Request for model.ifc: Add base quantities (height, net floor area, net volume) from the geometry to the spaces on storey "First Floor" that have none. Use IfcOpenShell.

First a look at what the model holds.

```python
import ifcopenshell
import ifcopenshell.util.element
import ifcopenshell.util.unit

model = ifcopenshell.open("model.ifc")
print(model.schema)
for unit_type in ("LENGTHUNIT", "AREAUNIT", "VOLUMEUNIT"):
    print(unit_type, ifcopenshell.util.unit.calculate_unit_scale(model, unit_type))
storey = next(s for s in model.by_type("IfcBuildingStorey") if s.Name == "First Floor")
spaces = [e for e in ifcopenshell.util.element.get_decomposition(storey) if e.is_a("IfcSpace")]
for e in sorted(spaces, key=lambda e: e.id()):
    print(e.id(), e.is_a(), e.Name, list(ifcopenshell.util.element.get_psets(e, qtos_only=True)), sep=" | ")
```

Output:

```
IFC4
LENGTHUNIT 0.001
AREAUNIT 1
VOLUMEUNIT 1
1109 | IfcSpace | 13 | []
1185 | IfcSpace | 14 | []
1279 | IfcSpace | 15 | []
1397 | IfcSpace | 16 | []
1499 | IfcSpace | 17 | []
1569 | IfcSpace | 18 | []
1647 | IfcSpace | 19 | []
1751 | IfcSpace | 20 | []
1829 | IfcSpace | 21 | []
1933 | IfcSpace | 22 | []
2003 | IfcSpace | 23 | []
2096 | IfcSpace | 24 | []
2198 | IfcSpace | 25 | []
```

```python
import ifcopenshell
import ifcopenshell.api.pset
import ifcopenshell.geom
import ifcopenshell.util.element
import ifcopenshell.util.shape
import ifcopenshell.util.unit

model = ifcopenshell.open("model.ifc")
unit_scale = ifcopenshell.util.unit.calculate_unit_scale(model)
area_scale = ifcopenshell.util.unit.calculate_unit_scale(model, "AREAUNIT")
volume_scale = ifcopenshell.util.unit.calculate_unit_scale(model, "VOLUMEUNIT")
settings = ifcopenshell.geom.settings()

storey = next(s for s in model.by_type("IfcBuildingStorey") if s.Name == "First Floor")
spaces = [e for e in ifcopenshell.util.element.get_decomposition(storey) if e.is_a("IfcSpace")]

for e in sorted(spaces, key=lambda e: e.id()):
    if ifcopenshell.util.element.get_psets(e, qtos_only=True, should_inherit=False):
        continue
    # Geometry comes back in metres, in the element's own axes.
    shape = ifcopenshell.geom.create_shape(settings, e)
    values = {
        "Height": ifcopenshell.util.shape.get_z(shape.geometry) / unit_scale,
        "NetFloorArea": ifcopenshell.util.shape.get_footprint_area(shape.geometry) / area_scale,
        "NetVolume": ifcopenshell.util.shape.get_volume(shape.geometry) / volume_scale,
    }
    qto = ifcopenshell.api.pset.add_qto(model, product=e, name="Qto_SpaceBaseQuantities")
    ifcopenshell.api.pset.edit_qto(model, qto=qto, properties=values)
    print(e.id(), {k: round(v, 3) for k, v in values.items()})

model.write("model_rev.ifc")
```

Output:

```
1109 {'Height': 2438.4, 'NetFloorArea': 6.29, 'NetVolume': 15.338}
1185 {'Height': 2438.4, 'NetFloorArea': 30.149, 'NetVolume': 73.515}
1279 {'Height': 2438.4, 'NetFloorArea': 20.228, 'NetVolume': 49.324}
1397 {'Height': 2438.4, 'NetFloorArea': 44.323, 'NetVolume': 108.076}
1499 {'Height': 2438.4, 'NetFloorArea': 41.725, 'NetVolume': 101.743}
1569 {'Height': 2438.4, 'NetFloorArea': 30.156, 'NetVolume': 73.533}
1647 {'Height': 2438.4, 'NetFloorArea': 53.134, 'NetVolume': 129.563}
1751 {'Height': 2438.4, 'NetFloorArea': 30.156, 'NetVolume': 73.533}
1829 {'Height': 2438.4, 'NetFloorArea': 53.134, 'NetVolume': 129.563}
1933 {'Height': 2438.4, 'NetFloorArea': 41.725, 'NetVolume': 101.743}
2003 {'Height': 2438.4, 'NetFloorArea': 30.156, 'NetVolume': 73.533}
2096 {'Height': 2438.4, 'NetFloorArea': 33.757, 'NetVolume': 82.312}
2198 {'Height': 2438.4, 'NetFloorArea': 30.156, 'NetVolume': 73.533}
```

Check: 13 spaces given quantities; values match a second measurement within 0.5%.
